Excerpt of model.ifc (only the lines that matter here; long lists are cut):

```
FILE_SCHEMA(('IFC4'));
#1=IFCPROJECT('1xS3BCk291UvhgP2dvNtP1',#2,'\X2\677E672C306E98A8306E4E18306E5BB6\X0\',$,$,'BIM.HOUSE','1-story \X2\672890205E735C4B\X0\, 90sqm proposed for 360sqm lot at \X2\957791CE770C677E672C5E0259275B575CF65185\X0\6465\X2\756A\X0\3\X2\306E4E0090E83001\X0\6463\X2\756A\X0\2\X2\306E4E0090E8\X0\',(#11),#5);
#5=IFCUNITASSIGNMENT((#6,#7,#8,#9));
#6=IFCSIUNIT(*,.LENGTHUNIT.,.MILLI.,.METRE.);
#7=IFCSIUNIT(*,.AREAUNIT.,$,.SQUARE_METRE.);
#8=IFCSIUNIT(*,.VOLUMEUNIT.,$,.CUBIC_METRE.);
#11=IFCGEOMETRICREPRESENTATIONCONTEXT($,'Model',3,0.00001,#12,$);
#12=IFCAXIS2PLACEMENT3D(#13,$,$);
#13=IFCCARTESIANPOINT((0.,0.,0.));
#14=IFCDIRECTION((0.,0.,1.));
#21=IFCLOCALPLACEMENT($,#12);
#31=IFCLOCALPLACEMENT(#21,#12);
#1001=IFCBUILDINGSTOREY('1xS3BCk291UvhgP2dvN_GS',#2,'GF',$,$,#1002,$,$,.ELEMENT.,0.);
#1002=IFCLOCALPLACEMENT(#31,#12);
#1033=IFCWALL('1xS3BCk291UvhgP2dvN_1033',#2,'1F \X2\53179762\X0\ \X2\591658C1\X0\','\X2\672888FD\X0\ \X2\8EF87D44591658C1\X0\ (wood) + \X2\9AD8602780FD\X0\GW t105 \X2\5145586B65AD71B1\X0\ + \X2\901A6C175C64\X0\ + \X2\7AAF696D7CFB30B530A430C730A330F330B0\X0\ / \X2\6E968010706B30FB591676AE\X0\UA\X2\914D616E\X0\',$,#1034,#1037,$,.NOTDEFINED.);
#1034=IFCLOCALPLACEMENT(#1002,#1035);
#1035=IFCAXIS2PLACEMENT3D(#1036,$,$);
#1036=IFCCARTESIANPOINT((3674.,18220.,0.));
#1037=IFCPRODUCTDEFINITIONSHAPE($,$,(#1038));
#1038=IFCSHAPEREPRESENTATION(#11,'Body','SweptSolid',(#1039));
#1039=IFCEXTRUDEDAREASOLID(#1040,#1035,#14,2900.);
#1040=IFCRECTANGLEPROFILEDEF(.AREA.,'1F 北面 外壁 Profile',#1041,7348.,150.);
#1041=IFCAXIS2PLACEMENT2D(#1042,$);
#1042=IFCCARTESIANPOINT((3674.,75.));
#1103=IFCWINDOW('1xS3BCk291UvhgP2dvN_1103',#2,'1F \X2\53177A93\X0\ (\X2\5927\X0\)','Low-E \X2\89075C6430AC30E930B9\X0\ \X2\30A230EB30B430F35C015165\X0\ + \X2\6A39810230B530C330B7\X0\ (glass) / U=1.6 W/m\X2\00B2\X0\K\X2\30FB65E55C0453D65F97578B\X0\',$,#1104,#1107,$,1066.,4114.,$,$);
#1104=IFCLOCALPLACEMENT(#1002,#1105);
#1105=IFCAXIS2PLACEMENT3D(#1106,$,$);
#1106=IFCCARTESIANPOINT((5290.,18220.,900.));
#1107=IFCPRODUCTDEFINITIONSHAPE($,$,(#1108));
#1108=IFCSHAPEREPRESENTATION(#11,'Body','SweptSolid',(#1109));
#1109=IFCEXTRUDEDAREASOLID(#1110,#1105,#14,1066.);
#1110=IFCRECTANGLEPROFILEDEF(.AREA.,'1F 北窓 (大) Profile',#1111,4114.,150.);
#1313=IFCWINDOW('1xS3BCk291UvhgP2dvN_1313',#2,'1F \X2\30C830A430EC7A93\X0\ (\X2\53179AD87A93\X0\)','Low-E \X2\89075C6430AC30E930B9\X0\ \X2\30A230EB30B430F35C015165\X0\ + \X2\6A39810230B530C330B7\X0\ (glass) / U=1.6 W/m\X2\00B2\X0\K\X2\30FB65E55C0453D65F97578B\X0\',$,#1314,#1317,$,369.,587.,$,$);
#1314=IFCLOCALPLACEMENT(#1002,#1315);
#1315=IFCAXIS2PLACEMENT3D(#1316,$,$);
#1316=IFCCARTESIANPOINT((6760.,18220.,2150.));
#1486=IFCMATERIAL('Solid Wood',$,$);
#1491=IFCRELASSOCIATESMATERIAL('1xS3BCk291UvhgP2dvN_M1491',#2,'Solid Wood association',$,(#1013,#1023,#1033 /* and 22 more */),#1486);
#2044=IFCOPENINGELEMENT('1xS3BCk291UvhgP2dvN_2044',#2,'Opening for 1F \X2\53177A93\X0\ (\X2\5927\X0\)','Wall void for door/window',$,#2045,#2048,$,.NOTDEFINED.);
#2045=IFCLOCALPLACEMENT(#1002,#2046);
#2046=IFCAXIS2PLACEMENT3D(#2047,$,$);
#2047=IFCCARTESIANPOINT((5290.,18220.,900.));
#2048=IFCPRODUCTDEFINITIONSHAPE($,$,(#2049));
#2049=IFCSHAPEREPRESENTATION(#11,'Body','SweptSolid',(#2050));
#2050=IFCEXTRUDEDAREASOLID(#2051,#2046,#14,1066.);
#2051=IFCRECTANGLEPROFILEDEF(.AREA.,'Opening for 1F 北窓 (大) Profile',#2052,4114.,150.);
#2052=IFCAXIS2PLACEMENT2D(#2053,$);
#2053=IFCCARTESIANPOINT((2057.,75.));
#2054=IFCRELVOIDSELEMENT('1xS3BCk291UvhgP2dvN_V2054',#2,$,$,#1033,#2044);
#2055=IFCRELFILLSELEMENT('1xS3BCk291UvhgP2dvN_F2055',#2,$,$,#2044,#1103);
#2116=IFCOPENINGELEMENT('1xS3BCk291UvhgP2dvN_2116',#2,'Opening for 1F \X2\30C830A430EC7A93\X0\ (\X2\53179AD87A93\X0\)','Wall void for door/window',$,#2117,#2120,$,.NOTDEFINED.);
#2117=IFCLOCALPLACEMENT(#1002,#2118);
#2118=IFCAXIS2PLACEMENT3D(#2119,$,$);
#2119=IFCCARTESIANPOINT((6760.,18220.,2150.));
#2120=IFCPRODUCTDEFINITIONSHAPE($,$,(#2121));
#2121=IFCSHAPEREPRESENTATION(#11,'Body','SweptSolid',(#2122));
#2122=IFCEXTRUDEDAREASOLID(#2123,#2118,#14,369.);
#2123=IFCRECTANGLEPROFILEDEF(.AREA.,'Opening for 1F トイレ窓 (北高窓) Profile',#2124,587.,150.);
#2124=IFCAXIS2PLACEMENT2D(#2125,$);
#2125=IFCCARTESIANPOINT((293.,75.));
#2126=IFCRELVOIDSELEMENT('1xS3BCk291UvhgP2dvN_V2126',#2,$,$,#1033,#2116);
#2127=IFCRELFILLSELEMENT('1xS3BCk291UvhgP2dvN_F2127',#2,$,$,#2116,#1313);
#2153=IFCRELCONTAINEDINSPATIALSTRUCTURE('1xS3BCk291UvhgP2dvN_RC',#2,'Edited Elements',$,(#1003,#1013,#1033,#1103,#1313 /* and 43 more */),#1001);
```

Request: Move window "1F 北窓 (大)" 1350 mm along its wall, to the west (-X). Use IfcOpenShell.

```python
import ifcopenshell
import ifcopenshell.api.geometry
import ifcopenshell.util.placement
import ifcopenshell.util.unit

model = ifcopenshell.open("model.ifc")
unit_scale = ifcopenshell.util.unit.calculate_unit_scale(model)

window = model.by_guid("1xS3BCk291UvhgP2dvN_1103")
opening = window.FillsVoids[0].RelatingOpeningElement
wall = opening.VoidsElements[0].RelatingBuildingElement

wall_matrix = ifcopenshell.util.placement.get_local_placement(wall.ObjectPlacement)
shift = wall_matrix[:3, 0] * -1.35 / unit_scale
before = ifcopenshell.util.placement.get_local_placement(window.ObjectPlacement)[:3, 3].copy()

# The window is not placed relative to its opening, so move both.
for product in (opening, window):
    matrix = ifcopenshell.util.placement.get_local_placement(product.ObjectPlacement)
    matrix[:3, 3] += shift
    ifcopenshell.api.geometry.edit_object_placement(model, product=product, matrix=matrix, is_si=False)

after = ifcopenshell.util.placement.get_local_placement(window.ObjectPlacement)[:3, 3]
print("window moved by", (after - before).round(3) + 0.0)

model.write("model_v2.ifc")
```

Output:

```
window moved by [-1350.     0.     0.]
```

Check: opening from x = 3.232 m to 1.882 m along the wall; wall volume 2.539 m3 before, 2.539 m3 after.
